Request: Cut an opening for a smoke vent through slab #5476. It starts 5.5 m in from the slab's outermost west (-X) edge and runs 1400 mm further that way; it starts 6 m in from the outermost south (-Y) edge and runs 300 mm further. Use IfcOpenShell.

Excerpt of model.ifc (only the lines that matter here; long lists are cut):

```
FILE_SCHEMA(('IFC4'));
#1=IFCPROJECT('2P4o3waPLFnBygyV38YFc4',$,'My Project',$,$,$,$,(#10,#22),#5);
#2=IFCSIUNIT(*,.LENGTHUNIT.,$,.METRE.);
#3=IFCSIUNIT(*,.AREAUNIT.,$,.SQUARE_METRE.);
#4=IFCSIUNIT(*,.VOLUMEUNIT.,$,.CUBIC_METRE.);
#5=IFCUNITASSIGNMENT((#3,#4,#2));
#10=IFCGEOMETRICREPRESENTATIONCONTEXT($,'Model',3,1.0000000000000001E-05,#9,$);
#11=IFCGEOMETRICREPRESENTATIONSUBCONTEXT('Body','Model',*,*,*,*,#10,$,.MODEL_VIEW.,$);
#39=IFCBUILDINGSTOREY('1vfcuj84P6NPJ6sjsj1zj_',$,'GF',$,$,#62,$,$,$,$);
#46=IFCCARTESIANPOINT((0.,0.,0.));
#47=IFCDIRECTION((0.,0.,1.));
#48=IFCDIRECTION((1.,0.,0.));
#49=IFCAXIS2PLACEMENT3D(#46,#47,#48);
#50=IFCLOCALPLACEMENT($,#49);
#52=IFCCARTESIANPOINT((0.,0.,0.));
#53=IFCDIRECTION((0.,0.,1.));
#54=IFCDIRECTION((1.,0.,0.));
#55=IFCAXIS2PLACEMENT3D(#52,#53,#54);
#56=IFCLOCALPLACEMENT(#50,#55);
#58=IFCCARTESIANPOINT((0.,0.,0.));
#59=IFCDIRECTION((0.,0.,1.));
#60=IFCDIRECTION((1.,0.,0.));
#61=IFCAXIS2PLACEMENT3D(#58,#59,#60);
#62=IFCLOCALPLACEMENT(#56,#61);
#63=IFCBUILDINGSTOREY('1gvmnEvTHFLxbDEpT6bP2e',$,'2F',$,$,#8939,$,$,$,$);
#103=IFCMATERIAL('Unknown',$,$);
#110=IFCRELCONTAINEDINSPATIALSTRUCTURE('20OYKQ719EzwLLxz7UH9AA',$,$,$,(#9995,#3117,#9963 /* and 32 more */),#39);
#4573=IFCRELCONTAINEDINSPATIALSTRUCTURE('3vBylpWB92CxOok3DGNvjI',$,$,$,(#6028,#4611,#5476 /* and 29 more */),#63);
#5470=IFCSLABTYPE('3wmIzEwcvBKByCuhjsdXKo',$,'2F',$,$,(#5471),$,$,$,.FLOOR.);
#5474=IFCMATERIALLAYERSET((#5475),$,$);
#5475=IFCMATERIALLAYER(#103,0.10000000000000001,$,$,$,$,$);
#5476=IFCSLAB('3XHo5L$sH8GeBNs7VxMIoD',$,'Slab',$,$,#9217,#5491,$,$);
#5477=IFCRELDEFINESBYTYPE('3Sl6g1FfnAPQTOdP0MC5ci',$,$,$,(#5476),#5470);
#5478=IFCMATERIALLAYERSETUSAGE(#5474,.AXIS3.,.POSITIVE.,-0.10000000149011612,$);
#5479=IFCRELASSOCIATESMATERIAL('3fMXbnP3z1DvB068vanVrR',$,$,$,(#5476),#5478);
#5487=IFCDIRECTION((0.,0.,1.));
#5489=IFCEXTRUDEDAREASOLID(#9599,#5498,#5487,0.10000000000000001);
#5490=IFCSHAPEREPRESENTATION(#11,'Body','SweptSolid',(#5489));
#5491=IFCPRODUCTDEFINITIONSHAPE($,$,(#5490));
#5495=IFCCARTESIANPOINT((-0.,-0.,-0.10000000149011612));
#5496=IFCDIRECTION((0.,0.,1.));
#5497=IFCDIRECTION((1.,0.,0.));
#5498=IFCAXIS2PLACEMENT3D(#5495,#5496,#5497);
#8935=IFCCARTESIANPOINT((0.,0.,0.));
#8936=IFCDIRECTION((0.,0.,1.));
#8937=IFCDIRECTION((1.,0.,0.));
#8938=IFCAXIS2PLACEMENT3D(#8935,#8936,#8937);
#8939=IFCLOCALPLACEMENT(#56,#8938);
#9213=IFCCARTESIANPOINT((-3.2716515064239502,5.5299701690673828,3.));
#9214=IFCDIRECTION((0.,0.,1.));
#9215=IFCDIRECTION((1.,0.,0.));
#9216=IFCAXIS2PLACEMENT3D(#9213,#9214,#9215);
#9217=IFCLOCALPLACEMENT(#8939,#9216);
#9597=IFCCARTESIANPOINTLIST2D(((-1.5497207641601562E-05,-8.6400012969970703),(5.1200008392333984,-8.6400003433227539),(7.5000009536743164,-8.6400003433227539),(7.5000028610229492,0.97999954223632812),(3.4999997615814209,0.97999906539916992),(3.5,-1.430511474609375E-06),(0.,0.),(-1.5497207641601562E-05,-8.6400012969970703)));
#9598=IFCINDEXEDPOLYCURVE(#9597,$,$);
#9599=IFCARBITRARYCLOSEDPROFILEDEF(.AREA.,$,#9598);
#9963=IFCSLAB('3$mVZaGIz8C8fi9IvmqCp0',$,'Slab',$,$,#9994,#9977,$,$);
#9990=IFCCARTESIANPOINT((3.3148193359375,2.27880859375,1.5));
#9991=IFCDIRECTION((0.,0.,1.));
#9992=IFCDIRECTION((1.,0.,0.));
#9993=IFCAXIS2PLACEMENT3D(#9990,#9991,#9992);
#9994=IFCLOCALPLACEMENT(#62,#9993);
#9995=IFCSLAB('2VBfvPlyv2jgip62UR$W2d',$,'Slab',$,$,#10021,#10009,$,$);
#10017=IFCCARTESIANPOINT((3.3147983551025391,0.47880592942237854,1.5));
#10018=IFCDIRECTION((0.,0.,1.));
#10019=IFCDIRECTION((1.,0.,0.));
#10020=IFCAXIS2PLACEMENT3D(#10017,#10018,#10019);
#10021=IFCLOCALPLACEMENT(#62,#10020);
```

```python
import numpy as np
import ifcopenshell
import ifcopenshell.api.feature
import ifcopenshell.api.geometry
import ifcopenshell.api.root
import ifcopenshell.geom
import ifcopenshell.util.placement
import ifcopenshell.util.representation
import ifcopenshell.util.shape
import ifcopenshell.util.unit

model = ifcopenshell.open("model.ifc")
unit_scale = ifcopenshell.util.unit.calculate_unit_scale(model)
settings = ifcopenshell.geom.settings()


def volume(element):
    """Net volume in cubic metres, openings subtracted."""
    shape = ifcopenshell.geom.create_shape(settings, element)
    return ifcopenshell.util.shape.get_volume(shape.geometry)


slab = model.by_guid("3XHo5L$sH8GeBNs7VxMIoD")
before = volume(slab)

# Extent in the slab's own axes, in metres. The edges named are its -X and -Y sides.
slab_shape = ifcopenshell.geom.create_shape(settings, slab)
vertices = ifcopenshell.util.shape.get_vertices(slab_shape.geometry)
x_min, y_min, bottom = vertices.min(axis=0)
top = vertices[:, 2].max()

opening = ifcopenshell.api.root.create_entity(model, ifc_class="IfcOpeningElement", name="Smoke vent opening", predefined_type="OPENING")
context = ifcopenshell.util.representation.get_context(model, "Model", "Body", "MODEL_VIEW")
width, depth = 1.4, 0.3
outline = [(0.0, 0.0), (width, 0.0), (width, depth), (0.0, depth), (0.0, 0.0)]
# Overshoot both faces by 50 mm so the cut is clean.
shape = ifcopenshell.api.geometry.add_slab_representation(
    model, context=context, depth=top - bottom + 0.1, polyline=outline
)
ifcopenshell.api.geometry.assign_representation(model, product=opening, representation=shape)

matrix = ifcopenshell.util.placement.get_local_placement(slab.ObjectPlacement)
matrix[:, 3] = matrix @ np.append(np.array([x_min + 5.5, y_min + 6, bottom - 0.05]) / unit_scale, 1.0)
ifcopenshell.api.geometry.edit_object_placement(model, product=opening, matrix=matrix, is_si=False)
ifcopenshell.api.feature.add_feature(model, feature=opening, element=slab)

after = volume(slab)

print(f"slab volume {before:.3f} -> {after:.3f} m3")

model.write("model_v2.ifc")
```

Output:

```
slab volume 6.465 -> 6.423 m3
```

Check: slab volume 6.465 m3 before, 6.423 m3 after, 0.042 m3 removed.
